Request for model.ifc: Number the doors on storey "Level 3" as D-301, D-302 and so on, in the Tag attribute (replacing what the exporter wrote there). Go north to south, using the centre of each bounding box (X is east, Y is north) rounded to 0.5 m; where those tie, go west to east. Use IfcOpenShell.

First a look at what the model holds.

```python
import ifcopenshell
import ifcopenshell.util.element
import ifcopenshell.util.placement

model = ifcopenshell.open("model.ifc")
print(model.schema)
storey = next(s for s in model.by_type("IfcBuildingStorey") if s.Name == "Level 3")
doors = [e for e in ifcopenshell.util.element.get_decomposition(storey) if e.is_a("IfcDoor")]
for e in sorted(doors, key=lambda e: e.id()):
    origin = ifcopenshell.util.placement.get_local_placement(e.ObjectPlacement)[:3, 3]
    print(e.id(), e.Tag, e.Name, origin.round(2) + 0.0, sep=" | ")
```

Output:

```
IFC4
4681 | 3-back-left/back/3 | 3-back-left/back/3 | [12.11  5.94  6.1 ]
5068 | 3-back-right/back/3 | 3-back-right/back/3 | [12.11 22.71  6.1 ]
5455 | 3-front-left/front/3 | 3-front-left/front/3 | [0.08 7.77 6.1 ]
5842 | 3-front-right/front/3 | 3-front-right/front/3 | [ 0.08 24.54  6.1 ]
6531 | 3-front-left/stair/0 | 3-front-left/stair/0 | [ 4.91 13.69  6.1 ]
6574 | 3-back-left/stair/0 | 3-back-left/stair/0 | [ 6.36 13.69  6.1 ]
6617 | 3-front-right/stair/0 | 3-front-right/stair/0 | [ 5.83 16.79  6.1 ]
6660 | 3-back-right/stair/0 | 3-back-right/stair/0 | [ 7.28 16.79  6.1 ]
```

```python
import ifcopenshell
import ifcopenshell.geom
import ifcopenshell.util.element
import ifcopenshell.util.shape

model = ifcopenshell.open("model.ifc")
settings = ifcopenshell.geom.settings()
settings.set("use-world-coords", True)


def centre(element):
    shape = ifcopenshell.geom.create_shape(settings, element)
    return ifcopenshell.util.shape.get_bbox_centroid(shape.geometry)


storey = next(s for s in model.by_type("IfcBuildingStorey") if s.Name == "Level 3")
doors = [e for e in ifcopenshell.util.element.get_decomposition(storey) if e.is_a("IfcDoor")]

# Insertion points can sit at a corner or the storey origin, so sort by the geometry (in metres).
centres = {e: centre(e) for e in doors}
doors.sort(key=lambda e: (-round(centres[e][1] / 0.5), centres[e][0]))

for i, e in enumerate(doors, start=1):
    number = f"D-3{i:02d}"
    e.Tag = number
    print(e.id(), number)

model.write("model_rev.ifc")
```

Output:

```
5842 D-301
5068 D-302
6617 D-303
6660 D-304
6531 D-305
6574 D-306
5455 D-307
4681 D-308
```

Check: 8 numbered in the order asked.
